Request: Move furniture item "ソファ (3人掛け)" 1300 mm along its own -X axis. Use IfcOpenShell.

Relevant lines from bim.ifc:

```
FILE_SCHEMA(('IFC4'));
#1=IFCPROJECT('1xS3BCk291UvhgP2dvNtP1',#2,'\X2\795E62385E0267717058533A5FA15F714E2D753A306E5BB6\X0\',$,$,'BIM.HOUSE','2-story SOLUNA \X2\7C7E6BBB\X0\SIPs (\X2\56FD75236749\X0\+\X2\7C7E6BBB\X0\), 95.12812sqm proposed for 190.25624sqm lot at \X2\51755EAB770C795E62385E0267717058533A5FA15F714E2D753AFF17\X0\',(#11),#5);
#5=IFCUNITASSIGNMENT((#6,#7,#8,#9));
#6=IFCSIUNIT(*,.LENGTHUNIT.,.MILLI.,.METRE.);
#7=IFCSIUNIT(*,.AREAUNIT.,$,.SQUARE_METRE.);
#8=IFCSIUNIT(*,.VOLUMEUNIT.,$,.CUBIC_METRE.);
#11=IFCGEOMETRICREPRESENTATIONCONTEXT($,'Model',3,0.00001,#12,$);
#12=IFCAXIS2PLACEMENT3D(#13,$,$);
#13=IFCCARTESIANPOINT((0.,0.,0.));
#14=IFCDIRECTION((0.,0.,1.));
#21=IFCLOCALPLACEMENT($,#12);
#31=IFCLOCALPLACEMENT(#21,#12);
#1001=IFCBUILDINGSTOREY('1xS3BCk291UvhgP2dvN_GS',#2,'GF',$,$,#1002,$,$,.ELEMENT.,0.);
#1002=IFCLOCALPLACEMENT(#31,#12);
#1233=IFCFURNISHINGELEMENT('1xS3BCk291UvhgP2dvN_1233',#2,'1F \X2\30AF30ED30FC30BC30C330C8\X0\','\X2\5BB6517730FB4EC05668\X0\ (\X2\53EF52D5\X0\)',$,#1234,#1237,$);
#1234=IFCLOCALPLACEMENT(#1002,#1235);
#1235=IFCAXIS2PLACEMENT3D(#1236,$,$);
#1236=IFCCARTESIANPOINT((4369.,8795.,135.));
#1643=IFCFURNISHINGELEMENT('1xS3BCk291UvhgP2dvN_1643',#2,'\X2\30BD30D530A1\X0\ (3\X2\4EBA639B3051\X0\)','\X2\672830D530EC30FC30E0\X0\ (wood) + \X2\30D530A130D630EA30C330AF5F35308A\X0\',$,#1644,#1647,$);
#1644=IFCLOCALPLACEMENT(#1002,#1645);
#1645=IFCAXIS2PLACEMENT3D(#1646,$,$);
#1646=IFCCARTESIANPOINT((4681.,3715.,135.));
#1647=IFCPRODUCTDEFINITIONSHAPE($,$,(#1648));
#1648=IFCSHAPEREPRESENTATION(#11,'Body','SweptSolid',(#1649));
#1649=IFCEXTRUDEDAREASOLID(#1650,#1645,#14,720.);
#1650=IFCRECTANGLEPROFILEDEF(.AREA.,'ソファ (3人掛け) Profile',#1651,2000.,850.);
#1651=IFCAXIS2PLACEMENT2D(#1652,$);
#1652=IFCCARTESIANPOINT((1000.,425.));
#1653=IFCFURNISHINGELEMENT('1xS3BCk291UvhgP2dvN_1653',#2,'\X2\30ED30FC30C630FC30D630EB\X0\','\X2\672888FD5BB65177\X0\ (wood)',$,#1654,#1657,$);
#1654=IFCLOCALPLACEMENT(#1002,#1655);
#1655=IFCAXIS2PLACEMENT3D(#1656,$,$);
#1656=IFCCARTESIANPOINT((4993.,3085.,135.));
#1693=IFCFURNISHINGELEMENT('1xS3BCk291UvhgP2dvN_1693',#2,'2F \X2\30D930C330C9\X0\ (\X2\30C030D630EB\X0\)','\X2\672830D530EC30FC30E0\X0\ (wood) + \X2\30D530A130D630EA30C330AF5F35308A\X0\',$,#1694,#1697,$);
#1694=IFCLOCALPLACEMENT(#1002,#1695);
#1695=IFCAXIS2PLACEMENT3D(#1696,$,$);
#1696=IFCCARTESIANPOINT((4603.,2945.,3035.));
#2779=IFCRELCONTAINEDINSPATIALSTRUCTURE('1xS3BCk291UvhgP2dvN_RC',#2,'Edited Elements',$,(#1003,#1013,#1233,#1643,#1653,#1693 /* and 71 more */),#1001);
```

```python
import ifcopenshell
import ifcopenshell.api.geometry
import ifcopenshell.util.placement
import ifcopenshell.util.unit

model = ifcopenshell.open("bim.ifc")
unit_scale = ifcopenshell.util.unit.calculate_unit_scale(model)

item = model.by_guid("1xS3BCk291UvhgP2dvN_1643")
matrix = ifcopenshell.util.placement.get_local_placement(item.ObjectPlacement)
matrix[:3, 3] -= matrix[:3, 0] * 1.3 / unit_scale
ifcopenshell.api.geometry.edit_object_placement(model, product=item, matrix=matrix, is_si=False)

print(ifcopenshell.util.placement.get_local_placement(item.ObjectPlacement).round(3) + 0.0)

model.write("bim_edited.ifc")
```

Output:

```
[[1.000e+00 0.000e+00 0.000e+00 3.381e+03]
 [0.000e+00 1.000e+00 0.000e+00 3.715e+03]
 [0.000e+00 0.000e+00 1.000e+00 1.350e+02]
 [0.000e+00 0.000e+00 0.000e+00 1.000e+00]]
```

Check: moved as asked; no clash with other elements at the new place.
